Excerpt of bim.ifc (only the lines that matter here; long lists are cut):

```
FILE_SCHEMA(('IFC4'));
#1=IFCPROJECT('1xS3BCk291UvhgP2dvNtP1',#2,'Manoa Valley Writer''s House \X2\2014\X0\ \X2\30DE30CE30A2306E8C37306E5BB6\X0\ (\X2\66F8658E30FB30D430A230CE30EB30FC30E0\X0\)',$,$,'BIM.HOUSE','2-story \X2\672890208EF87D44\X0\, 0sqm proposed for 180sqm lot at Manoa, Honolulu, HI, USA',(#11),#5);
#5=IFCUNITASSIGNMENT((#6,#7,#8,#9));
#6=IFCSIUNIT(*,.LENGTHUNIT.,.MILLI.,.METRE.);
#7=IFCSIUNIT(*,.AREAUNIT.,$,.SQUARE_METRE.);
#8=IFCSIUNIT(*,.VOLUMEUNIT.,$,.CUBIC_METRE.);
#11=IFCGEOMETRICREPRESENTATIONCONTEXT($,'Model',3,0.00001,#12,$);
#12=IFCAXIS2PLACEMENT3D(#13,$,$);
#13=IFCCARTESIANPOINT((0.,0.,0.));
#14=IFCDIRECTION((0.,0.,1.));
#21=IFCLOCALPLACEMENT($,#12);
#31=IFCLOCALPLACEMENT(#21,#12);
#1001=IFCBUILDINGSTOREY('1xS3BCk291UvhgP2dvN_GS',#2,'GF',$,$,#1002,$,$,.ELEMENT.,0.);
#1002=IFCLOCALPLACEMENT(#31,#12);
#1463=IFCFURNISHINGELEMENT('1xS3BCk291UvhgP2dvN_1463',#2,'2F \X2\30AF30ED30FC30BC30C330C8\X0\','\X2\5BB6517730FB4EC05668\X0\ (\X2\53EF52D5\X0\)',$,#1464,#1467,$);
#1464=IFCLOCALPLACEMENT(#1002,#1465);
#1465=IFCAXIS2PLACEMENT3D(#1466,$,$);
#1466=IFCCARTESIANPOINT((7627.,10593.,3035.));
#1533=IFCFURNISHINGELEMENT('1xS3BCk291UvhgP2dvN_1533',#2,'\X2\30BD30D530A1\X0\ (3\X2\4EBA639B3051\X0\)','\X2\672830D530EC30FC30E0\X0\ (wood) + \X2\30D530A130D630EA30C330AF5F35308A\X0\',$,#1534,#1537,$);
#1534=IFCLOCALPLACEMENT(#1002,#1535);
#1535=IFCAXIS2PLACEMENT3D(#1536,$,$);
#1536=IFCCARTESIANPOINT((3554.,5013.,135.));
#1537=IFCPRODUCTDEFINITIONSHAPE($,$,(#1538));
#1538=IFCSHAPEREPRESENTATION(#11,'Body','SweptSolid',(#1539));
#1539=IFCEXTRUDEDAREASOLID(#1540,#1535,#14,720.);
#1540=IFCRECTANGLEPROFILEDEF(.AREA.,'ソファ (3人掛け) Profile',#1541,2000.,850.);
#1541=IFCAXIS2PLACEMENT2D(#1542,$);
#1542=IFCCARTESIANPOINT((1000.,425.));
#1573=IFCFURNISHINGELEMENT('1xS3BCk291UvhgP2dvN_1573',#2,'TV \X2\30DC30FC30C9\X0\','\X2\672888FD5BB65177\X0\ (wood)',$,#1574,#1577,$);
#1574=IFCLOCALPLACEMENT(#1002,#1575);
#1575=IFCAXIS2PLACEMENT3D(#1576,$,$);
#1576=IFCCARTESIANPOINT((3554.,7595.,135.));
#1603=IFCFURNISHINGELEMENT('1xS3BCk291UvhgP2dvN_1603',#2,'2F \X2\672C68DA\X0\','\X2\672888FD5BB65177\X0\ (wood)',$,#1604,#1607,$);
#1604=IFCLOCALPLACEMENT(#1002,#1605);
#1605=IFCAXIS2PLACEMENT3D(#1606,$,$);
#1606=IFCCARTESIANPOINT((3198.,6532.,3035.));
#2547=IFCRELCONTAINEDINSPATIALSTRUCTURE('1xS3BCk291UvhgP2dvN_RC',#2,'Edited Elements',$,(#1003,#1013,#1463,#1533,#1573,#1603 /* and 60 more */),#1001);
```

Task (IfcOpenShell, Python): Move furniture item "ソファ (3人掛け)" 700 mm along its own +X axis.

```python
import ifcopenshell
import ifcopenshell.api.geometry
import ifcopenshell.util.placement
import ifcopenshell.util.unit

model = ifcopenshell.open("bim.ifc")
unit_scale = ifcopenshell.util.unit.calculate_unit_scale(model)

item = model.by_id(1533)
matrix = ifcopenshell.util.placement.get_local_placement(item.ObjectPlacement)
matrix[:3, 3] += matrix[:3, 0] * 0.7 / unit_scale
ifcopenshell.api.geometry.edit_object_placement(model, product=item, matrix=matrix, is_si=False)

print(ifcopenshell.util.placement.get_local_placement(item.ObjectPlacement).round(3) + 0.0)

model.write("bim_edited.ifc")
```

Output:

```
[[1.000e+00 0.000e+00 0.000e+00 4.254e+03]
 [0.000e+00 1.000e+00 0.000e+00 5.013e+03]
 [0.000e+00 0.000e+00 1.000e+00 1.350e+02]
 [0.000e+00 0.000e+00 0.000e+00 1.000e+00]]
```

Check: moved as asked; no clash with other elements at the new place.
